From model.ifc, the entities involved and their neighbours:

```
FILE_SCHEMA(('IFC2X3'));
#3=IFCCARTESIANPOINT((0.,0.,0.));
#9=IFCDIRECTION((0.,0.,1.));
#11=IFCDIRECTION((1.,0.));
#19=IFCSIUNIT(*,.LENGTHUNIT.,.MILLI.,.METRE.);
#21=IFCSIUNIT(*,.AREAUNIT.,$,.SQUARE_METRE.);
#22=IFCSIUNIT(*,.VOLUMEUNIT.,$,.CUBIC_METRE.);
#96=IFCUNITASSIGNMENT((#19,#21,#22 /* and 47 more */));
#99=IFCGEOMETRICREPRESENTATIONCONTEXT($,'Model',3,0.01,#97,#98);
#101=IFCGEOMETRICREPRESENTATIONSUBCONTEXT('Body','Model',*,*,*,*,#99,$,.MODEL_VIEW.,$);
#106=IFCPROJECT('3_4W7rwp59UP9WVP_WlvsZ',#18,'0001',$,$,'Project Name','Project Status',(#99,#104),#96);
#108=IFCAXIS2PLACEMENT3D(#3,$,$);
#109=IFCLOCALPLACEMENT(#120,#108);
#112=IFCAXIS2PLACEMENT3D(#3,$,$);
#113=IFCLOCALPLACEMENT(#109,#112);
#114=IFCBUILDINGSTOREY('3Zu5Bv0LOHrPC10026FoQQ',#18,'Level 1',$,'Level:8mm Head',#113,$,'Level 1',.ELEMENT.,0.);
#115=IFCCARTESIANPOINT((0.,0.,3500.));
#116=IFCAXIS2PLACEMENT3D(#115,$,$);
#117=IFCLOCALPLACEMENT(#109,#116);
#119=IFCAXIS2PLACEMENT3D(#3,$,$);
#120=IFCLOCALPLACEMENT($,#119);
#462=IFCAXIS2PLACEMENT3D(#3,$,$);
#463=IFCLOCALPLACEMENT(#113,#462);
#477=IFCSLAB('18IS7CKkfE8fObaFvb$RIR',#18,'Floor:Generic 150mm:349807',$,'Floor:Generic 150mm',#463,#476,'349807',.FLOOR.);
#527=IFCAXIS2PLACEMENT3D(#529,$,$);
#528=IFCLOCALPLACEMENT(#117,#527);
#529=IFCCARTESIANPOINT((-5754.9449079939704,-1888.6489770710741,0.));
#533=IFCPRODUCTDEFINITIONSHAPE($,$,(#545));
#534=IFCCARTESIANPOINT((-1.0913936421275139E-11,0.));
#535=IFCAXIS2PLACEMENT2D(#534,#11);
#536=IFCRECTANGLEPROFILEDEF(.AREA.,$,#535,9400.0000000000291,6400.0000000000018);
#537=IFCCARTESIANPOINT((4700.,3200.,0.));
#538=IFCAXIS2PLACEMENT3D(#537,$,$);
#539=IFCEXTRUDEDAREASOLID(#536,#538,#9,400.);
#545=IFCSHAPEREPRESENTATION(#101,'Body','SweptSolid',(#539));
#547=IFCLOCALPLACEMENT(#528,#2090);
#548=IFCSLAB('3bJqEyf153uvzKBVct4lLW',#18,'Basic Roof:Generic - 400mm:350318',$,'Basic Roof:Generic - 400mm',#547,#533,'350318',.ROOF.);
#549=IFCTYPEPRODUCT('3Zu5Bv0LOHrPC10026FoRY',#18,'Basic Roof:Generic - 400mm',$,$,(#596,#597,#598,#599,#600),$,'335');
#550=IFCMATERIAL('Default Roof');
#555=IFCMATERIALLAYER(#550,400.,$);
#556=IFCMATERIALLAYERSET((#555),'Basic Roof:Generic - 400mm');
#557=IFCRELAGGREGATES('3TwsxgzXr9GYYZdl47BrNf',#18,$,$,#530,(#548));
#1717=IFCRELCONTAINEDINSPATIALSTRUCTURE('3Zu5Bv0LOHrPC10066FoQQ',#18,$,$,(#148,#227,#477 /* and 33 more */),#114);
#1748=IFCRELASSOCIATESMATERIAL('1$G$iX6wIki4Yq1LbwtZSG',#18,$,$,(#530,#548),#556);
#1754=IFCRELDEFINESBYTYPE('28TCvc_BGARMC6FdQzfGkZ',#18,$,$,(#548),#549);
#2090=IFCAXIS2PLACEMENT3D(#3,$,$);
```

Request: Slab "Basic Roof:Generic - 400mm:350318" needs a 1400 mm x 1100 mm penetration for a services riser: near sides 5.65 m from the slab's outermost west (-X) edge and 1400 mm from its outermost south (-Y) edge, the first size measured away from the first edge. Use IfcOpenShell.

```python
import numpy as np
import ifcopenshell
import ifcopenshell.api.feature
import ifcopenshell.api.geometry
import ifcopenshell.api.root
import ifcopenshell.geom
import ifcopenshell.util.placement
import ifcopenshell.util.representation
import ifcopenshell.util.shape
import ifcopenshell.util.unit

model = ifcopenshell.open("model.ifc")
unit_scale = ifcopenshell.util.unit.calculate_unit_scale(model)
settings = ifcopenshell.geom.settings()


def volume(element):
    """Net volume in cubic metres, openings subtracted."""
    shape = ifcopenshell.geom.create_shape(settings, element)
    return ifcopenshell.util.shape.get_volume(shape.geometry)


slab = model.by_guid("3bJqEyf153uvzKBVct4lLW")
before = volume(slab)

# Extent in the slab's own axes, in metres. The edges named are its -X and -Y sides.
slab_shape = ifcopenshell.geom.create_shape(settings, slab)
vertices = ifcopenshell.util.shape.get_vertices(slab_shape.geometry)
x_min, y_min, bottom = vertices.min(axis=0)
top = vertices[:, 2].max()

opening = ifcopenshell.api.root.create_entity(model, ifc_class="IfcOpeningElement", name="Services riser opening")
context = ifcopenshell.util.representation.get_context(model, "Model", "Body", "MODEL_VIEW")
width, depth = 1.4, 1.1
outline = [(0.0, 0.0), (width, 0.0), (width, depth), (0.0, depth), (0.0, 0.0)]
# Overshoot both faces by 50 mm so the cut is clean.
shape = ifcopenshell.api.geometry.add_slab_representation(
    model, context=context, depth=top - bottom + 0.1, polyline=outline
)
ifcopenshell.api.geometry.assign_representation(model, product=opening, representation=shape)

matrix = ifcopenshell.util.placement.get_local_placement(slab.ObjectPlacement)
matrix[:, 3] = matrix @ np.append(np.array([x_min + 5.65, y_min + 1.4, bottom - 0.05]) / unit_scale, 1.0)
ifcopenshell.api.geometry.edit_object_placement(model, product=opening, matrix=matrix, is_si=False)
ifcopenshell.api.feature.add_feature(model, feature=opening, element=slab)

after = volume(slab)

print(f"slab volume {before:.3f} -> {after:.3f} m3")

model.write("model_updated.ifc")
```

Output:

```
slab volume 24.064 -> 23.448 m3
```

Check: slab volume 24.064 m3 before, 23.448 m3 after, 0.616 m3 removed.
